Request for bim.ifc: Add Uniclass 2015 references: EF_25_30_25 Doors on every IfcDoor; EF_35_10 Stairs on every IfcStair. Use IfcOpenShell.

First a look at what the model holds.

```python
import ifcopenshell

model = ifcopenshell.open("bim.ifc")
print(model.schema)
print("classifications:", [c.Name for c in model.by_type("IfcClassification")])
for ifc_class in ("IfcDoor", "IfcRoof", "IfcStair", "IfcWall", "IfcWindow"):
    print(ifc_class, len(model.by_type(ifc_class)))
```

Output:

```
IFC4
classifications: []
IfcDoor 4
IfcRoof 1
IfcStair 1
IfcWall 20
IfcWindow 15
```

```python
import ifcopenshell
import ifcopenshell.api.classification

model = ifcopenshell.open("bim.ifc")

system = ifcopenshell.api.classification.add_classification(model, classification="Uniclass 2015")

codes = {
    "IfcDoor": ("EF_25_30_25", "Doors"),
    "IfcStair": ("EF_35_10", "Stairs"),
}
for ifc_class, (code, name) in codes.items():
    products = model.by_type(ifc_class)
    ifcopenshell.api.classification.add_reference(
        model, products=products, classification=system, identification=code, name=name
    )
    print(code, len(products))

model.write("bim_edited.ifc")
```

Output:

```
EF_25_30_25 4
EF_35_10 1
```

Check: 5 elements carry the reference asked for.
